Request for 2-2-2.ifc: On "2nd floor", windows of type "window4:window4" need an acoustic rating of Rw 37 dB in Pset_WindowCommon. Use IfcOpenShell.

First a look at what the model holds.

```python
import ifcopenshell
import ifcopenshell.util.element

model = ifcopenshell.open("2-2-2.ifc")
print(model.schema)
storey = next(s for s in model.by_type("IfcBuildingStorey") if s.Name == "2nd floor")
windows = [e for e in ifcopenshell.util.element.get_decomposition(storey) if e.is_a("IfcWindow")]
seen = {}
for e in windows:
    element_type = ifcopenshell.util.element.get_type(e)
    key = (element_type.Name if element_type != e and element_type else None, ifcopenshell.util.element.get_pset(e, "Pset_WindowCommon", "AcousticRating"))
    seen[key] = seen.get(key, 0) + 1
for (name, value), count in sorted(seen.items(), key=str):
    print(count, "x", name, "|", value)
```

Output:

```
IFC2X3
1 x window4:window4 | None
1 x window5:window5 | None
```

```python
import ifcopenshell
import ifcopenshell.api.pset
import ifcopenshell.util.element

model = ifcopenshell.open("2-2-2.ifc")

storey = next(s for s in model.by_type("IfcBuildingStorey") if s.Name == "2nd floor")
windows = [e for e in ifcopenshell.util.element.get_decomposition(storey) if e.is_a("IfcWindow")]

count = 0
for e in windows:
    element_type = ifcopenshell.util.element.get_type(e)
    if element_type in (None, e) or element_type.Name != "window4:window4":
        continue
    # add_pset returns the element's existing set when there is one.
    pset = ifcopenshell.api.pset.add_pset(model, product=e, name="Pset_WindowCommon")
    ifcopenshell.api.pset.edit_pset(model, pset=pset, properties={"AcousticRating": "Rw 37 dB"})
    count += 1

print(count, "windows updated")

model.write("2-2-2_v2.ifc")
```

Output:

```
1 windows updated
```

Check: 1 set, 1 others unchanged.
